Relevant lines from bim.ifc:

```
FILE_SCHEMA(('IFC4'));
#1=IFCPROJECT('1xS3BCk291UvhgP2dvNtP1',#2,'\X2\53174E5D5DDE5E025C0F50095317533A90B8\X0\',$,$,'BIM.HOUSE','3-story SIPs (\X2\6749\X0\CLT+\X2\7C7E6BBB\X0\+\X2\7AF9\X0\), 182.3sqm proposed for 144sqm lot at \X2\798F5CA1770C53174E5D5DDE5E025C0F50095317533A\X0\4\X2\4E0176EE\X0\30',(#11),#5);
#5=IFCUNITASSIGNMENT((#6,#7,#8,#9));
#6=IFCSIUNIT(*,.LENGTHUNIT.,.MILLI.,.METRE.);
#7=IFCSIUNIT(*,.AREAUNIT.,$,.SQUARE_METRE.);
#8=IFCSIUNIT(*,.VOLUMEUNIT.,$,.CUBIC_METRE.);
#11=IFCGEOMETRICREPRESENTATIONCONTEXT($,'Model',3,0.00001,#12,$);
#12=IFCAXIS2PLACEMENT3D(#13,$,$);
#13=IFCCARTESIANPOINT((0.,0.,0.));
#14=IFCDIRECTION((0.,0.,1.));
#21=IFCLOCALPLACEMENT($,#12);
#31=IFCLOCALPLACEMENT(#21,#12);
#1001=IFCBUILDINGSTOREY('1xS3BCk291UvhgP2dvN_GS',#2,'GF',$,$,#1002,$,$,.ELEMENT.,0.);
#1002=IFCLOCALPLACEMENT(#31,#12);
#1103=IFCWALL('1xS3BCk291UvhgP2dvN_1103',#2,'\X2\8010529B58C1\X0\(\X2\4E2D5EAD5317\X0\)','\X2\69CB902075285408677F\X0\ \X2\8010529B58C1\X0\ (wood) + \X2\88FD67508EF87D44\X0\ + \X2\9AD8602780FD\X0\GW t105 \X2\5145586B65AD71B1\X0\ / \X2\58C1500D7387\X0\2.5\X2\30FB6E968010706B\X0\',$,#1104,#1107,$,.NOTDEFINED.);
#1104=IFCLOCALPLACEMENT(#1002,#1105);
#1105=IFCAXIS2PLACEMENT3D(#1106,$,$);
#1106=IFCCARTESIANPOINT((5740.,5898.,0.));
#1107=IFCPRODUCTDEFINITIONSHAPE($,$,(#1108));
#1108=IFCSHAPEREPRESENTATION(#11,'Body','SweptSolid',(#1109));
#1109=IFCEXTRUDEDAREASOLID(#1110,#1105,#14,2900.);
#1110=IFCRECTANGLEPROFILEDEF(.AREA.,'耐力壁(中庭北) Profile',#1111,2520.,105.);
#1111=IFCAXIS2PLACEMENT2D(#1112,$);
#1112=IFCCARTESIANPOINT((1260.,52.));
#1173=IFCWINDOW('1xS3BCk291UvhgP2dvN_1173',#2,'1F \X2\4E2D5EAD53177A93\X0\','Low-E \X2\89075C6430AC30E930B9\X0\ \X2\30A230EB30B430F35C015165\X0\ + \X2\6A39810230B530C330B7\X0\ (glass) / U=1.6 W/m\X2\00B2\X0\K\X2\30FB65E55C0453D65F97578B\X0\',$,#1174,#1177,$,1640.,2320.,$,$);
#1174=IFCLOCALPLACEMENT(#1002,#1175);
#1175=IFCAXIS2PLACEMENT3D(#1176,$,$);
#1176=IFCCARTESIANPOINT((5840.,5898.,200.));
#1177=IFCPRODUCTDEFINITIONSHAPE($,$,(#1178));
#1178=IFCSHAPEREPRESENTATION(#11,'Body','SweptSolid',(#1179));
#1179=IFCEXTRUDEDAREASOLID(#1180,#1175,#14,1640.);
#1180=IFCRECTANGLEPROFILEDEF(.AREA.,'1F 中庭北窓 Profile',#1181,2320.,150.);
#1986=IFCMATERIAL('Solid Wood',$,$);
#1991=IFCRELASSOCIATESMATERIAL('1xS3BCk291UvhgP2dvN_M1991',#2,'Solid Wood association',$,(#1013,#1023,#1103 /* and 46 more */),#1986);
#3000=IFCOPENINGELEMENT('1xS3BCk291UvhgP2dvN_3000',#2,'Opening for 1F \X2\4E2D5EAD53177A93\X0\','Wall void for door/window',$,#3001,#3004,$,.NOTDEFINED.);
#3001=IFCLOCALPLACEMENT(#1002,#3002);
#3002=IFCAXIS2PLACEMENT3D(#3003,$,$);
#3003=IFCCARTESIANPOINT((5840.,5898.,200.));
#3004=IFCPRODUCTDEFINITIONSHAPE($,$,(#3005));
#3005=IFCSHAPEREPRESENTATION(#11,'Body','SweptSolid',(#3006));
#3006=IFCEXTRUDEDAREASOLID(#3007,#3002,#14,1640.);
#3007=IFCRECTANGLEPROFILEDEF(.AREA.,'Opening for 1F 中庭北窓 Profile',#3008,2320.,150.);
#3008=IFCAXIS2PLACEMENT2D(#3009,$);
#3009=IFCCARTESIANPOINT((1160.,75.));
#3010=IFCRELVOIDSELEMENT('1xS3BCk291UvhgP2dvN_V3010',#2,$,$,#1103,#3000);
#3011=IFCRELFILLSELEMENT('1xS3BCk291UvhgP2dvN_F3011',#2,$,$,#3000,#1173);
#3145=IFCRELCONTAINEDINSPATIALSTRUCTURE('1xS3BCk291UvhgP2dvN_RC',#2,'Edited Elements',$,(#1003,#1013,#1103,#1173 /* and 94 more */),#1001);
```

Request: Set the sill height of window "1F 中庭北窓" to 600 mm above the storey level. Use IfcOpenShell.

```python
import numpy as np
import ifcopenshell
import ifcopenshell.api.geometry
import ifcopenshell.geom
import ifcopenshell.util.element
import ifcopenshell.util.placement
import ifcopenshell.util.shape
import ifcopenshell.util.unit

model = ifcopenshell.open("bim.ifc")
unit_scale = ifcopenshell.util.unit.calculate_unit_scale(model)

window = model.by_guid("1xS3BCk291UvhgP2dvN_1173")
opening = window.FillsVoids[0].RelatingOpeningElement
storey = ifcopenshell.util.element.get_container(window, ifc_class="IfcBuildingStorey")
level = ifcopenshell.util.placement.get_local_placement(storey.ObjectPlacement)[2, 3]

# The opening's origin need not be at the sill, so measure its lowest point.
shape = ifcopenshell.geom.create_shape(ifcopenshell.geom.settings(), opening)
bottom = ifcopenshell.util.shape.get_shape_bottom_elevation(shape, shape.geometry) / unit_scale
dz = level + 0.6 / unit_scale - bottom

shift = np.array([0.0, 0.0, dz])
# The window is not placed relative to its opening, so move both.
for product in (opening, window):
    matrix = ifcopenshell.util.placement.get_local_placement(product.ObjectPlacement)
    matrix[:3, 3] += shift
    ifcopenshell.api.geometry.edit_object_placement(model, product=product, matrix=matrix, is_si=False)

print(f"moved by {dz * unit_scale:+.3f} m")

model.write("bim-out.ifc")
```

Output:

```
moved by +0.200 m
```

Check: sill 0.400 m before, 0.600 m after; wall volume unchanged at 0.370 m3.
